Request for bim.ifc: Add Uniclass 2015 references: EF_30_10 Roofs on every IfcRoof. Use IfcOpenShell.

First a look at what the model holds.

```python
import ifcopenshell

model = ifcopenshell.open("bim.ifc")
print(model.schema)
print("classifications:", [c.Name for c in model.by_type("IfcClassification")])
for ifc_class in ("IfcDoor", "IfcRoof", "IfcStair", "IfcWall", "IfcWindow"):
    print(ifc_class, len(model.by_type(ifc_class)))
```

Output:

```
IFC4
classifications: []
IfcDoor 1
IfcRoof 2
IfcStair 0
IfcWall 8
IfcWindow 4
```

```python
import ifcopenshell
import ifcopenshell.api.classification

model = ifcopenshell.open("bim.ifc")

system = ifcopenshell.api.classification.add_classification(model, classification="Uniclass 2015")

codes = {
    "IfcRoof": ("EF_30_10", "Roofs"),
}
for ifc_class, (code, name) in codes.items():
    products = model.by_type(ifc_class)
    ifcopenshell.api.classification.add_reference(
        model, products=products, classification=system, identification=code, name=name
    )
    print(code, len(products))

model.write("bim_rev.ifc")
```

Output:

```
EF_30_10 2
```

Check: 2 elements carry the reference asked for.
